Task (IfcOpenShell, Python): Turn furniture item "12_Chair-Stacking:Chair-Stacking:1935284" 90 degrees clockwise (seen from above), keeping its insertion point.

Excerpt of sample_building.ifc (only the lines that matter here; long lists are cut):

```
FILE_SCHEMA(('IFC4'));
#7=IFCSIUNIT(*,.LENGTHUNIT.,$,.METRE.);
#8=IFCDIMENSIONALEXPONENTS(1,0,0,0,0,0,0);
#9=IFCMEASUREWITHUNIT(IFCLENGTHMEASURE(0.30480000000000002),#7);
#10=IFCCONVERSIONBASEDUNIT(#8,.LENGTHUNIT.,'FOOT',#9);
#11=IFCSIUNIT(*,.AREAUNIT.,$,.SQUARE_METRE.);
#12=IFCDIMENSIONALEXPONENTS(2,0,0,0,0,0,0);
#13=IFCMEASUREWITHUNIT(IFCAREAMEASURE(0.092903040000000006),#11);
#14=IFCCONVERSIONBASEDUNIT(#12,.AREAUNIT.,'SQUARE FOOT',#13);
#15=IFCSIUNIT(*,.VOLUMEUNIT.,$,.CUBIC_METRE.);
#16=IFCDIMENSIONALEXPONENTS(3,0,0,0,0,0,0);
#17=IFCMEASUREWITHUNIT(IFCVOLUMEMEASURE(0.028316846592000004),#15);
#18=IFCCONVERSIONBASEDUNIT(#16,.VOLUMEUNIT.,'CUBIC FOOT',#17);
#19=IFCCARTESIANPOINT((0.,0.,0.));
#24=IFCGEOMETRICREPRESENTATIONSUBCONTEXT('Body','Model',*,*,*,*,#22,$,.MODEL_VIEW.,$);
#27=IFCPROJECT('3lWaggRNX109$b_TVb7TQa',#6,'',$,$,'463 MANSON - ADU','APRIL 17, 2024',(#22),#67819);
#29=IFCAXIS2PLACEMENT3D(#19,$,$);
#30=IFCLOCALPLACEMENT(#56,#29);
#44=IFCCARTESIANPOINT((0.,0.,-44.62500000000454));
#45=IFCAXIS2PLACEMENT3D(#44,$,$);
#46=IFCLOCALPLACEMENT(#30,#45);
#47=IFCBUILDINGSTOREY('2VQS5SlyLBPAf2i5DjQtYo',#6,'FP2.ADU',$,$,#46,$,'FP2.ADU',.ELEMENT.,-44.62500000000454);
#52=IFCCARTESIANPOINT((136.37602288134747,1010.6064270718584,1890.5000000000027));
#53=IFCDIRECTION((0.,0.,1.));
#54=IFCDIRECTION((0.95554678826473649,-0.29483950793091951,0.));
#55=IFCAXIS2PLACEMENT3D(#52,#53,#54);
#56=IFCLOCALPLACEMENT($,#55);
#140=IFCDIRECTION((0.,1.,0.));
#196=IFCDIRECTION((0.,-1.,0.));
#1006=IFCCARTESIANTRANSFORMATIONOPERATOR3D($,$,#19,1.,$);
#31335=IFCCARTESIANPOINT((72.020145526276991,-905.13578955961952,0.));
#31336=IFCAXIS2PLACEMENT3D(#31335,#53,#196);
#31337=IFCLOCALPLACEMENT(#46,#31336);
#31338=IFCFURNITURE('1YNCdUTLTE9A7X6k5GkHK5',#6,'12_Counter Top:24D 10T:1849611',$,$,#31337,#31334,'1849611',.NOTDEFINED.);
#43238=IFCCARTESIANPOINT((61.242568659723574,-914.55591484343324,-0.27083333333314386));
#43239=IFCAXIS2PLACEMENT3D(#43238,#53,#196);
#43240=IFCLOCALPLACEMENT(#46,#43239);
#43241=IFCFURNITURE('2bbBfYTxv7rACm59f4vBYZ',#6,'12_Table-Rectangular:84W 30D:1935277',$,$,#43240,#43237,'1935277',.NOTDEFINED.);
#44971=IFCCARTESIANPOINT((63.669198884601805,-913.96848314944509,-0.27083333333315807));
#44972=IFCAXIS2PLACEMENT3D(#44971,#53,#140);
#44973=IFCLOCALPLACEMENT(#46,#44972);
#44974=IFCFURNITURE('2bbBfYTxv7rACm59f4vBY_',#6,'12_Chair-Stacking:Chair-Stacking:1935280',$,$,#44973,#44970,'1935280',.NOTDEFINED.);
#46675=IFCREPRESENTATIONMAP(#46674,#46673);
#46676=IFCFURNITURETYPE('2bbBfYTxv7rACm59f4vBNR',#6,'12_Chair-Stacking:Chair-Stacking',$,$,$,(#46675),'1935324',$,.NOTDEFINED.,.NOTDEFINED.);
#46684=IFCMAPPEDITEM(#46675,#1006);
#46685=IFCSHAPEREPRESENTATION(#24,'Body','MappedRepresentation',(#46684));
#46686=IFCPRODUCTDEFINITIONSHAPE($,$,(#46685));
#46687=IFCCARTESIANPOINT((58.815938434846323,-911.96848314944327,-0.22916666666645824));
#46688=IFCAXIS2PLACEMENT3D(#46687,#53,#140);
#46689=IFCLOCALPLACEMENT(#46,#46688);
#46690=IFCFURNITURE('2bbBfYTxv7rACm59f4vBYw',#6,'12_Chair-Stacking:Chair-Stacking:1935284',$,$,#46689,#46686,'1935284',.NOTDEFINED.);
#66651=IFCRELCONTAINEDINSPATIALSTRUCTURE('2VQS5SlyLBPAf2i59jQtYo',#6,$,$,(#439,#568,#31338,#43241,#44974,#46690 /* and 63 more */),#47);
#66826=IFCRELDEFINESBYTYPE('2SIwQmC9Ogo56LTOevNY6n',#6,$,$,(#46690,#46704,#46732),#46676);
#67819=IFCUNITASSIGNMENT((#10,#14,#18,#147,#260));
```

```python
import ifcopenshell
import ifcopenshell.api.geometry
import ifcopenshell.util.placement

model = ifcopenshell.open("sample_building.ifc")

item = model.by_guid("2bbBfYTxv7rACm59f4vBYw")
matrix = ifcopenshell.util.placement.get_local_placement(item.ObjectPlacement)
matrix = matrix @ ifcopenshell.util.placement.rotation(-90, "Z")
ifcopenshell.api.geometry.edit_object_placement(model, product=item, matrix=matrix, is_si=False)

print(ifcopenshell.util.placement.get_local_placement(item.ObjectPlacement).round(3) + 0.0)

model.write("sample_building_edited.ifc")
```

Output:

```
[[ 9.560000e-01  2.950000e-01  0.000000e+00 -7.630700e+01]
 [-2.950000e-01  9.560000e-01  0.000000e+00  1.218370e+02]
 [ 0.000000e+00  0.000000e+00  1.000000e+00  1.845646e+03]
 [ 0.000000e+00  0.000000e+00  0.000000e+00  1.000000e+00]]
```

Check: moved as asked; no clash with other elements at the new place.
